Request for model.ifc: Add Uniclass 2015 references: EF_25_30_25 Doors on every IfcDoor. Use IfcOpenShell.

First a look at what the model holds.

```python
import ifcopenshell

model = ifcopenshell.open("model.ifc")
print(model.schema)
print("classifications:", [c.Name for c in model.by_type("IfcClassification")])
for ifc_class in ("IfcDoor", "IfcRoof", "IfcStair", "IfcWall", "IfcWindow"):
    print(ifc_class, len(model.by_type(ifc_class)))
```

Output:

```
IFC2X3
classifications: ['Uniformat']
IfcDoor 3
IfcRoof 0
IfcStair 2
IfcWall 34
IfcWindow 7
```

```python
import ifcopenshell
import ifcopenshell.api.classification

model = ifcopenshell.open("model.ifc")

# IFC2X3 requires Source and Edition and has no link from the project to the system.
system = model.create_entity("IfcClassification", Source="NBS", Edition="2015", Name="Uniclass 2015")

codes = {
    "IfcDoor": ("EF_25_30_25", "Doors"),
}
for ifc_class, (code, name) in codes.items():
    products = model.by_type(ifc_class)
    ifcopenshell.api.classification.add_reference(
        model, products=products, classification=system, identification=code, name=name
    )
    print(code, len(products))

model.write("model_updated.ifc")
```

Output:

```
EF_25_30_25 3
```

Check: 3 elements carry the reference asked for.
